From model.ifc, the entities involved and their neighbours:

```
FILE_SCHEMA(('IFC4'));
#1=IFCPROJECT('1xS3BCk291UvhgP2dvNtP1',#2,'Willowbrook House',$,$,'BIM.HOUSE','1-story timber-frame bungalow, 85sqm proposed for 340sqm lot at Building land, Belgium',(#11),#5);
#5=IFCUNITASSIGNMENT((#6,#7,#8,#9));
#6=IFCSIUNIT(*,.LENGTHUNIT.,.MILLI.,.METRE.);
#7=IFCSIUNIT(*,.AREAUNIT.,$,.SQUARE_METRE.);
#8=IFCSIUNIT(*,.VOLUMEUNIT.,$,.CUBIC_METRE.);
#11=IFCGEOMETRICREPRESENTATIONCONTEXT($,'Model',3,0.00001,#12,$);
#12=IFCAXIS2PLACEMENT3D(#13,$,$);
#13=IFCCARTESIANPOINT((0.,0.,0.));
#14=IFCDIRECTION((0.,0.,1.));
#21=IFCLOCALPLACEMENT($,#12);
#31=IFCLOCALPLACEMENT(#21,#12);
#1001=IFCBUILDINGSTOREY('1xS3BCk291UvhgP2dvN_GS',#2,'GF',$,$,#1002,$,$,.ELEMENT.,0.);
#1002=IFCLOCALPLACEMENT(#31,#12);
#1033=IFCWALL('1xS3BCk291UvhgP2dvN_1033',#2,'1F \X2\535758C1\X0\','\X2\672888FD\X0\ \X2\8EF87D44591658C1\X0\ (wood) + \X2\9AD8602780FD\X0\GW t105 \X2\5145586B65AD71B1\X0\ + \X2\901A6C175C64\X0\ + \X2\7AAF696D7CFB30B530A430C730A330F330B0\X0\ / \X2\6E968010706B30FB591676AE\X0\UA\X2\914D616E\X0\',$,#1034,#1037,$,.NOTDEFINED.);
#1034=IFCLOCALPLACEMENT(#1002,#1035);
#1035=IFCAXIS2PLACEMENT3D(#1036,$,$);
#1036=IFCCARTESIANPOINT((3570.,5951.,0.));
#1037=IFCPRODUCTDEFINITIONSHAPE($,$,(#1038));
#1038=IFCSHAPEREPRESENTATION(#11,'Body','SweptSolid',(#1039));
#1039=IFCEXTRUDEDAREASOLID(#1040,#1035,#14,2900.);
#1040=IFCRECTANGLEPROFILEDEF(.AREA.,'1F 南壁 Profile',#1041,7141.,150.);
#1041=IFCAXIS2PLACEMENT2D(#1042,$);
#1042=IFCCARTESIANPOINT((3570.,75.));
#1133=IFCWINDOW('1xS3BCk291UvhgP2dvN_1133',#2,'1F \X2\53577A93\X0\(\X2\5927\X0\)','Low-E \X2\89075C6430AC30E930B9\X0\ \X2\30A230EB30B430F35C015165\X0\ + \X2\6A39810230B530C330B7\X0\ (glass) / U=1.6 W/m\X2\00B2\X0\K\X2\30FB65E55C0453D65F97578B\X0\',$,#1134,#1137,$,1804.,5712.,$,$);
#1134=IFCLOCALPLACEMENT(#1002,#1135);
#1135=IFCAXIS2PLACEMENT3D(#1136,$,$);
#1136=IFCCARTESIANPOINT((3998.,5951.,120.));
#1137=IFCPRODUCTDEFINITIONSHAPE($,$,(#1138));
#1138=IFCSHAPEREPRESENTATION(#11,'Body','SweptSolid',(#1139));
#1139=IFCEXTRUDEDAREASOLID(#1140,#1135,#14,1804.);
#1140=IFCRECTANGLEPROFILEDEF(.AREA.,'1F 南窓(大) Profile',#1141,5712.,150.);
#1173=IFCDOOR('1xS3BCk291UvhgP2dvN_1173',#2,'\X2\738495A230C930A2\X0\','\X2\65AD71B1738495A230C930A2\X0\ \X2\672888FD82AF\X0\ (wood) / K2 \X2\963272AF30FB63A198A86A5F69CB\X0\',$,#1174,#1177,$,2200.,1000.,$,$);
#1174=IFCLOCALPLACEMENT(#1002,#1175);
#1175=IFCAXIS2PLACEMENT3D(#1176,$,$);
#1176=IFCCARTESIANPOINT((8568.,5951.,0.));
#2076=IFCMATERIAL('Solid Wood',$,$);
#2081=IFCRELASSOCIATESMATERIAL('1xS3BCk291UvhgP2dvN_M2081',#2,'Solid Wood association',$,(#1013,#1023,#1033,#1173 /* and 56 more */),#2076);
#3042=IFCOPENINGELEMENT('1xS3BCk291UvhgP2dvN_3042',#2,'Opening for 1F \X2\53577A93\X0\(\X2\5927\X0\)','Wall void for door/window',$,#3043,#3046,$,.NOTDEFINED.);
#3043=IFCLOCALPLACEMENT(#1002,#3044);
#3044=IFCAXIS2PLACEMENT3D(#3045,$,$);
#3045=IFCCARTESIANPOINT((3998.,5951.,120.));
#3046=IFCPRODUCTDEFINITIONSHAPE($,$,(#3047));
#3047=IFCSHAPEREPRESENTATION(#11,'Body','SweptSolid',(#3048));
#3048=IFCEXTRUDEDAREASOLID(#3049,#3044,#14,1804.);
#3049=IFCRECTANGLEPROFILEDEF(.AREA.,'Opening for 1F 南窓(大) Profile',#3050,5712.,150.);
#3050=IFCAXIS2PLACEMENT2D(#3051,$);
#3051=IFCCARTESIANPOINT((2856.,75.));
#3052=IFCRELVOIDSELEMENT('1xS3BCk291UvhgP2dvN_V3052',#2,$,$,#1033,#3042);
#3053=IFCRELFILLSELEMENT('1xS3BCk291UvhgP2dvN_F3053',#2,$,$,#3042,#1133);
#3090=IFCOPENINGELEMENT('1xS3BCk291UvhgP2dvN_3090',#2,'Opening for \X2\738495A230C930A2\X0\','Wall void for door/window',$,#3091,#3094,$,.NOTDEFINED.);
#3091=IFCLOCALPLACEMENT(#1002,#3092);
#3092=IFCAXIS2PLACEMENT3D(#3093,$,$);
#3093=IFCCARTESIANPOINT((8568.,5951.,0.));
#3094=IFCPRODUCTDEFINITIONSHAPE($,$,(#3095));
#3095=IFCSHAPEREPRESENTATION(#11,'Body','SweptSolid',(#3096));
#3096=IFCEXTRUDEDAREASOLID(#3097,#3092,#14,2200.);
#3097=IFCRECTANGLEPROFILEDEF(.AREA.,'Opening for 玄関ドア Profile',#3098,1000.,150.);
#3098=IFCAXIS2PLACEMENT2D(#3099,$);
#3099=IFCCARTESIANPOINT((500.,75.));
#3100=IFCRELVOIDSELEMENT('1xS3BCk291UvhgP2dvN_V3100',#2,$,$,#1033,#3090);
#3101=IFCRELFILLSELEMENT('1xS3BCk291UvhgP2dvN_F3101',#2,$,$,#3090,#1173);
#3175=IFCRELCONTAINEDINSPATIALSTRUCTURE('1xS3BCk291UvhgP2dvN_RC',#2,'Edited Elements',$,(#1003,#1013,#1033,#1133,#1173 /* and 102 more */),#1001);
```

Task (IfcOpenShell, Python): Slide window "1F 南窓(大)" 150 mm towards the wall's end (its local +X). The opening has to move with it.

```python
import ifcopenshell
import ifcopenshell.api.geometry
import ifcopenshell.util.placement

model = ifcopenshell.open("model.ifc")

window = model.by_guid("1xS3BCk291UvhgP2dvN_1133")
opening = window.FillsVoids[0].RelatingOpeningElement
wall = opening.VoidsElements[0].RelatingBuildingElement

wall_matrix = ifcopenshell.util.placement.get_local_placement(wall.ObjectPlacement)
shift = wall_matrix[:3, 0] * 150.0
before = ifcopenshell.util.placement.get_local_placement(window.ObjectPlacement)[:3, 3].copy()

# The window is not placed relative to its opening, so move both.
for product in (opening, window):
    matrix = ifcopenshell.util.placement.get_local_placement(product.ObjectPlacement)
    matrix[:3, 3] += shift
    ifcopenshell.api.geometry.edit_object_placement(model, product=product, matrix=matrix, is_si=False)

after = ifcopenshell.util.placement.get_local_placement(window.ObjectPlacement)[:3, 3]
print("window moved by", (after - before).round(3) + 0.0)

model.write("model-out.ifc")
```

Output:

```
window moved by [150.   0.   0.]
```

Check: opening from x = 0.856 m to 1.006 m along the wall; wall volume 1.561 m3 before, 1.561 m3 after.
